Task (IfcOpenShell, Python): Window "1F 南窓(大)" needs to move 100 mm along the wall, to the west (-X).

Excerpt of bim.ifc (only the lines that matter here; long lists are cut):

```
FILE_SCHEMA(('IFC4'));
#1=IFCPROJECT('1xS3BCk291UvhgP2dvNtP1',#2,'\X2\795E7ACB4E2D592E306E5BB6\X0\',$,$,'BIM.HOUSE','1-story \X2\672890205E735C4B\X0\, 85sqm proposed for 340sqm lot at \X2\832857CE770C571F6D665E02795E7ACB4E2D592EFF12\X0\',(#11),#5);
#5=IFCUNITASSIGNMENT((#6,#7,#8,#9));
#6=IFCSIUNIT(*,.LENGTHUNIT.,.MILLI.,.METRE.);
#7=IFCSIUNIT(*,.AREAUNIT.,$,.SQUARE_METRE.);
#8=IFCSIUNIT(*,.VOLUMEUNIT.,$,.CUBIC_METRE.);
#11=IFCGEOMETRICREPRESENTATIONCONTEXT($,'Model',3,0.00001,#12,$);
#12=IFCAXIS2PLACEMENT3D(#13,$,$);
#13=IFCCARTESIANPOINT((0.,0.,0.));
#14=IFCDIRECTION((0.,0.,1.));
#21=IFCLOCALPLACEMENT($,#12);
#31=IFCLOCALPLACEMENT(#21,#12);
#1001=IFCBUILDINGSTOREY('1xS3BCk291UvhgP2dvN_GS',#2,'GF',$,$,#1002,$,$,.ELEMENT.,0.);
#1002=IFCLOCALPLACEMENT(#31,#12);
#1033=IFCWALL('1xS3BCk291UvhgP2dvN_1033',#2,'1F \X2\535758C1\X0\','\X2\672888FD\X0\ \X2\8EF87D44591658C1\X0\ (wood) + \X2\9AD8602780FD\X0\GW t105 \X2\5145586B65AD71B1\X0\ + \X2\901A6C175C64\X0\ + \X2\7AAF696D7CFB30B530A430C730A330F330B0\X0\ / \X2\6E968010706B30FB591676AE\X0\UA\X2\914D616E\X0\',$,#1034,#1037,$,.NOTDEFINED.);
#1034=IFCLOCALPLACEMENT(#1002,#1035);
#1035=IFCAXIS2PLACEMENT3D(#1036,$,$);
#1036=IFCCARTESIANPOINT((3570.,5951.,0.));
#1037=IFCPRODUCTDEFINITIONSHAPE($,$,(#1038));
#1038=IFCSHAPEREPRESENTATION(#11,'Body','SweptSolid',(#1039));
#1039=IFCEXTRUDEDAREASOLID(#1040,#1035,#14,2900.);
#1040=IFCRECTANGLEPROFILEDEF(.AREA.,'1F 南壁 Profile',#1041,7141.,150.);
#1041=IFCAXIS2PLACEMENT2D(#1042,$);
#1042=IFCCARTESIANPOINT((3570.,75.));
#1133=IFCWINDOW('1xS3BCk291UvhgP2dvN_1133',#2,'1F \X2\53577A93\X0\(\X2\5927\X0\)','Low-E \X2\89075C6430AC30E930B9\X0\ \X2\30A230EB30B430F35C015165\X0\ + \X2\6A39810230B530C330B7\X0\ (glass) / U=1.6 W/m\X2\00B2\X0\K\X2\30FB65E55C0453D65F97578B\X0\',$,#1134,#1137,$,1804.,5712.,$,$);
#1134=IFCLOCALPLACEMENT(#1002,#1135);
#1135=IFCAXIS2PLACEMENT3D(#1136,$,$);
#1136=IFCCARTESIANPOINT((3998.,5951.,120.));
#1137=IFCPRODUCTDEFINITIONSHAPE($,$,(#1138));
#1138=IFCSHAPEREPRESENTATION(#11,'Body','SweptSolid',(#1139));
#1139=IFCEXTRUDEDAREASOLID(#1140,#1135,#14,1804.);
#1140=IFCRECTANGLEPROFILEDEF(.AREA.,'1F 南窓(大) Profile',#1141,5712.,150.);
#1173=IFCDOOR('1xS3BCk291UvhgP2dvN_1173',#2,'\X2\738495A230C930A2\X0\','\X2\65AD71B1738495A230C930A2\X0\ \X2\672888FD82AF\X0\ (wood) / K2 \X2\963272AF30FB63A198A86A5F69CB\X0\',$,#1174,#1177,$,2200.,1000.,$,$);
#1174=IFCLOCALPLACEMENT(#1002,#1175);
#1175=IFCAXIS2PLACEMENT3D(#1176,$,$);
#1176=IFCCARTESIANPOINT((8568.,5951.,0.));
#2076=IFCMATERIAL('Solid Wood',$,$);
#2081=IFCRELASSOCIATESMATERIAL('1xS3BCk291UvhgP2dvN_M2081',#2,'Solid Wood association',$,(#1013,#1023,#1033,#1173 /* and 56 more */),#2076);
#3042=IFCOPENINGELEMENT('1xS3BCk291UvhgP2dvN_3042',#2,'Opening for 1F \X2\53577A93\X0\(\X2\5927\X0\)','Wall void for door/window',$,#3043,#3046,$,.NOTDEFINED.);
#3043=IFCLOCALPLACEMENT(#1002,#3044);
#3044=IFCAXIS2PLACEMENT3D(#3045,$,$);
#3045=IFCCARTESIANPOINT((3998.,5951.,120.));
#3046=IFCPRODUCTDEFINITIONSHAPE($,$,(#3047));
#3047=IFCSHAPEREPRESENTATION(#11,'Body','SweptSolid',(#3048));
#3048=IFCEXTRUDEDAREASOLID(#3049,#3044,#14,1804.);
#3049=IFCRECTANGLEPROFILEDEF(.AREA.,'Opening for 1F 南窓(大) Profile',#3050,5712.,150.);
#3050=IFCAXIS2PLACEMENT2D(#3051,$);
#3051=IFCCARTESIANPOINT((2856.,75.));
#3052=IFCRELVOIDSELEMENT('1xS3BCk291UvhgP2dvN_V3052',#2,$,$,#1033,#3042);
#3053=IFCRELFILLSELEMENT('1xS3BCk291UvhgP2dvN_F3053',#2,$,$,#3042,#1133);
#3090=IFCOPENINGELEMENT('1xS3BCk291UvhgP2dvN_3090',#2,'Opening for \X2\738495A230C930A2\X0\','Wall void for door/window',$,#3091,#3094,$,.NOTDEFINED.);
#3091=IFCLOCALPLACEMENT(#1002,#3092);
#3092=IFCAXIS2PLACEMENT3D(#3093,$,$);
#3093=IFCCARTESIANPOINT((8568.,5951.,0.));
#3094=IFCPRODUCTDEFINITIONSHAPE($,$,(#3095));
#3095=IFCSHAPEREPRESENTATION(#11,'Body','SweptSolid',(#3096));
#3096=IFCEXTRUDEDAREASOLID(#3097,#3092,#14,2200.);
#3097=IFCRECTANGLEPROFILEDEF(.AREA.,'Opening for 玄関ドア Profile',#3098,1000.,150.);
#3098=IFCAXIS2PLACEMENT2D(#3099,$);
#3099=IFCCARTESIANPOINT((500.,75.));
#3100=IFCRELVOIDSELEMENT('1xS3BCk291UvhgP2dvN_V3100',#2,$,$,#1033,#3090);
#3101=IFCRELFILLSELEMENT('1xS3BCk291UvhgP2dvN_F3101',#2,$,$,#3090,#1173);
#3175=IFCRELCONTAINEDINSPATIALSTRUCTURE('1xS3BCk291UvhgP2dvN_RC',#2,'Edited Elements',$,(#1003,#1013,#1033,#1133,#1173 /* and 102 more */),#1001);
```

```python
import ifcopenshell
import ifcopenshell.api.geometry
import ifcopenshell.util.placement
import ifcopenshell.util.unit

model = ifcopenshell.open("bim.ifc")
unit_scale = ifcopenshell.util.unit.calculate_unit_scale(model)

window = model.by_guid("1xS3BCk291UvhgP2dvN_1133")
opening = window.FillsVoids[0].RelatingOpeningElement
wall = opening.VoidsElements[0].RelatingBuildingElement

wall_matrix = ifcopenshell.util.placement.get_local_placement(wall.ObjectPlacement)
shift = wall_matrix[:3, 0] * -0.1 / unit_scale
before = ifcopenshell.util.placement.get_local_placement(window.ObjectPlacement)[:3, 3].copy()

# The window is not placed relative to its opening, so move both.
for product in (opening, window):
    matrix = ifcopenshell.util.placement.get_local_placement(product.ObjectPlacement)
    matrix[:3, 3] += shift
    ifcopenshell.api.geometry.edit_object_placement(model, product=product, matrix=matrix, is_si=False)

after = ifcopenshell.util.placement.get_local_placement(window.ObjectPlacement)[:3, 3]
print("window moved by", (after - before).round(3) + 0.0)

model.write("bim_updated.ifc")
```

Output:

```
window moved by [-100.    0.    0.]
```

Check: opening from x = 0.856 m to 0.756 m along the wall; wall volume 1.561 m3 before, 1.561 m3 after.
